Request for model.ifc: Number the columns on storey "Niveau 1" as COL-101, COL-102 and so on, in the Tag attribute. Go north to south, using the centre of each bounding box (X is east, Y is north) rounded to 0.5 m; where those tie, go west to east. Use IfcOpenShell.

First a look at what the model holds.

```python
import ifcopenshell
import ifcopenshell.util.element
import ifcopenshell.util.placement

model = ifcopenshell.open("model.ifc")
print(model.schema)
storey = next(s for s in model.by_type("IfcBuildingStorey") if s.Name == "Niveau 1")
columns = [e for e in ifcopenshell.util.element.get_decomposition(storey) if e.is_a("IfcColumn")]
for e in sorted(columns, key=lambda e: e.id()):
    origin = ifcopenshell.util.placement.get_local_placement(e.ObjectPlacement)[:3, 3]
    print(e.id(), e.Tag, e.Name, origin.round(2) + 0.0, sep=" | ")
```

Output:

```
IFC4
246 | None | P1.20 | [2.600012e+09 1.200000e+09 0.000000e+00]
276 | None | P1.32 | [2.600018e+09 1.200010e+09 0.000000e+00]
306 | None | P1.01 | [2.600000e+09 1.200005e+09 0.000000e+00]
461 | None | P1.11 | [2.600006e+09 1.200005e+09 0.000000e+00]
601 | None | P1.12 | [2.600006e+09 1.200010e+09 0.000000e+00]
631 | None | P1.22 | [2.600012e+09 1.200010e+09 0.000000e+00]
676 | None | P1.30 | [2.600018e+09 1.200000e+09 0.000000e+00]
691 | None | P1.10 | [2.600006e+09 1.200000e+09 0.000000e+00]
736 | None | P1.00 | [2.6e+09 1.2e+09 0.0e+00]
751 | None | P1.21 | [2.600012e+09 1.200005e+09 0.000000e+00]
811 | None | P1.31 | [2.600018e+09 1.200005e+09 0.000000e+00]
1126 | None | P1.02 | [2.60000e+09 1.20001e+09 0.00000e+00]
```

```python
import ifcopenshell
import ifcopenshell.geom
import ifcopenshell.util.element
import ifcopenshell.util.shape

model = ifcopenshell.open("model.ifc")
settings = ifcopenshell.geom.settings()
settings.set("use-world-coords", True)


def centre(element):
    shape = ifcopenshell.geom.create_shape(settings, element)
    return ifcopenshell.util.shape.get_bbox_centroid(shape.geometry)


storey = next(s for s in model.by_type("IfcBuildingStorey") if s.Name == "Niveau 1")
columns = [e for e in ifcopenshell.util.element.get_decomposition(storey) if e.is_a("IfcColumn")]

# Insertion points can sit at a corner or the storey origin, so sort by the geometry (in metres).
centres = {e: centre(e) for e in columns}
columns.sort(key=lambda e: (-round(centres[e][1] / 0.5), centres[e][0]))

for i, e in enumerate(columns, start=1):
    number = f"COL-1{i:02d}"
    e.Tag = number
    print(e.id(), number)

model.write("model-out.ifc")
```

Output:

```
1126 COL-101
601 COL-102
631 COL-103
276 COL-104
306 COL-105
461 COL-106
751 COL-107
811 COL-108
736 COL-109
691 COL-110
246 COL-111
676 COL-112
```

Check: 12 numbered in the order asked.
